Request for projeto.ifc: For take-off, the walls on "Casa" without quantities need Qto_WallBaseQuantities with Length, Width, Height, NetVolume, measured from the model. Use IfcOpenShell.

First a look at what the model holds.

```python
import ifcopenshell
import ifcopenshell.util.element
import ifcopenshell.util.unit

model = ifcopenshell.open("projeto.ifc")
print(model.schema)
for unit_type in ("LENGTHUNIT", "AREAUNIT", "VOLUMEUNIT"):
    print(unit_type, ifcopenshell.util.unit.calculate_unit_scale(model, unit_type))
storey = next(s for s in model.by_type("IfcBuildingStorey") if s.Name == "Casa")
walls = [e for e in ifcopenshell.util.element.get_decomposition(storey) if e.is_a("IfcWall")]
for e in sorted(walls, key=lambda e: e.id()):
    print(e.id(), e.is_a(), e.Name, list(ifcopenshell.util.element.get_psets(e, qtos_only=True)), sep=" | ")
```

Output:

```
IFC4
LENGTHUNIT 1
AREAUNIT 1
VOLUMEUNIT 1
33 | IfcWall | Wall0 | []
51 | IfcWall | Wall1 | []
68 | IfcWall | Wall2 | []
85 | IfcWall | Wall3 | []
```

```python
import ifcopenshell
import ifcopenshell.api.pset
import ifcopenshell.geom
import ifcopenshell.util.element
import ifcopenshell.util.shape
import ifcopenshell.util.unit

model = ifcopenshell.open("projeto.ifc")
unit_scale = ifcopenshell.util.unit.calculate_unit_scale(model)
volume_scale = ifcopenshell.util.unit.calculate_unit_scale(model, "VOLUMEUNIT")
settings = ifcopenshell.geom.settings()

storey = next(s for s in model.by_type("IfcBuildingStorey") if s.Name == "Casa")
walls = [e for e in ifcopenshell.util.element.get_decomposition(storey) if e.is_a("IfcWall")]

for e in sorted(walls, key=lambda e: e.id()):
    if ifcopenshell.util.element.get_psets(e, qtos_only=True, should_inherit=False):
        continue
    # Geometry comes back in metres, in the element's own axes.
    shape = ifcopenshell.geom.create_shape(settings, e)
    values = {
        "Length": ifcopenshell.util.shape.get_x(shape.geometry) / unit_scale,
        "Width": ifcopenshell.util.shape.get_y(shape.geometry) / unit_scale,
        "Height": ifcopenshell.util.shape.get_z(shape.geometry) / unit_scale,
        "NetVolume": ifcopenshell.util.shape.get_volume(shape.geometry) / volume_scale,
    }
    qto = ifcopenshell.api.pset.add_qto(model, product=e, name="Qto_WallBaseQuantities")
    ifcopenshell.api.pset.edit_qto(model, qto=qto, properties=values)
    print(e.id(), {k: round(v, 3) for k, v in values.items()})

model.write("projeto_edited.ifc")
```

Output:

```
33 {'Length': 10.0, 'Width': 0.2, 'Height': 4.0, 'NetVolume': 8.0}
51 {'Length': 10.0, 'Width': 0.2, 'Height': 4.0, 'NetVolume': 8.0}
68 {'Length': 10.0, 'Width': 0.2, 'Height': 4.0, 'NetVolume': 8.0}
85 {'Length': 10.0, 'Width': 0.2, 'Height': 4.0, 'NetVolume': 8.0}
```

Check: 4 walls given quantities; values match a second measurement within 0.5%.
